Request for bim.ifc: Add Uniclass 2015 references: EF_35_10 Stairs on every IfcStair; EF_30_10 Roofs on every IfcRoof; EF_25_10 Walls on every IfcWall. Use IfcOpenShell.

First a look at what the model holds.

```python
import ifcopenshell

model = ifcopenshell.open("bim.ifc")
print(model.schema)
print("classifications:", [c.Name for c in model.by_type("IfcClassification")])
for ifc_class in ("IfcDoor", "IfcRoof", "IfcStair", "IfcWall", "IfcWindow"):
    print(ifc_class, len(model.by_type(ifc_class)))
```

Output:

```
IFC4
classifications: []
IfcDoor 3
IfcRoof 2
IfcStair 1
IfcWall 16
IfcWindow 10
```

```python
import ifcopenshell
import ifcopenshell.api.classification

model = ifcopenshell.open("bim.ifc")

system = ifcopenshell.api.classification.add_classification(model, classification="Uniclass 2015")

codes = {
    "IfcStair": ("EF_35_10", "Stairs"),
    "IfcRoof": ("EF_30_10", "Roofs"),
    "IfcWall": ("EF_25_10", "Walls"),
}
for ifc_class, (code, name) in codes.items():
    products = model.by_type(ifc_class)
    ifcopenshell.api.classification.add_reference(
        model, products=products, classification=system, identification=code, name=name
    )
    print(code, len(products))

model.write("bim_rev.ifc")
```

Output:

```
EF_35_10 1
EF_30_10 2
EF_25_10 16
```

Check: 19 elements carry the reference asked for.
